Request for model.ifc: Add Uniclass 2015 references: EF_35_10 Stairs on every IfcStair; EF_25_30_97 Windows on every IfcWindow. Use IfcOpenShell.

First a look at what the model holds.

```python
import ifcopenshell

model = ifcopenshell.open("model.ifc")
print(model.schema)
print("classifications:", [c.Name for c in model.by_type("IfcClassification")])
for ifc_class in ("IfcDoor", "IfcRoof", "IfcStair", "IfcWall", "IfcWindow"):
    print(ifc_class, len(model.by_type(ifc_class)))
```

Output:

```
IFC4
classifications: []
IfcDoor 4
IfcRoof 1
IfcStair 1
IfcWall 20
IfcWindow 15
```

```python
import ifcopenshell
import ifcopenshell.api.classification

model = ifcopenshell.open("model.ifc")

system = ifcopenshell.api.classification.add_classification(model, classification="Uniclass 2015")

codes = {
    "IfcStair": ("EF_35_10", "Stairs"),
    "IfcWindow": ("EF_25_30_97", "Windows"),
}
for ifc_class, (code, name) in codes.items():
    products = model.by_type(ifc_class)
    ifcopenshell.api.classification.add_reference(
        model, products=products, classification=system, identification=code, name=name
    )
    print(code, len(products))

model.write("model_edited.ifc")
```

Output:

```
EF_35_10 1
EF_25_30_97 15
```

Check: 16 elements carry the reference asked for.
